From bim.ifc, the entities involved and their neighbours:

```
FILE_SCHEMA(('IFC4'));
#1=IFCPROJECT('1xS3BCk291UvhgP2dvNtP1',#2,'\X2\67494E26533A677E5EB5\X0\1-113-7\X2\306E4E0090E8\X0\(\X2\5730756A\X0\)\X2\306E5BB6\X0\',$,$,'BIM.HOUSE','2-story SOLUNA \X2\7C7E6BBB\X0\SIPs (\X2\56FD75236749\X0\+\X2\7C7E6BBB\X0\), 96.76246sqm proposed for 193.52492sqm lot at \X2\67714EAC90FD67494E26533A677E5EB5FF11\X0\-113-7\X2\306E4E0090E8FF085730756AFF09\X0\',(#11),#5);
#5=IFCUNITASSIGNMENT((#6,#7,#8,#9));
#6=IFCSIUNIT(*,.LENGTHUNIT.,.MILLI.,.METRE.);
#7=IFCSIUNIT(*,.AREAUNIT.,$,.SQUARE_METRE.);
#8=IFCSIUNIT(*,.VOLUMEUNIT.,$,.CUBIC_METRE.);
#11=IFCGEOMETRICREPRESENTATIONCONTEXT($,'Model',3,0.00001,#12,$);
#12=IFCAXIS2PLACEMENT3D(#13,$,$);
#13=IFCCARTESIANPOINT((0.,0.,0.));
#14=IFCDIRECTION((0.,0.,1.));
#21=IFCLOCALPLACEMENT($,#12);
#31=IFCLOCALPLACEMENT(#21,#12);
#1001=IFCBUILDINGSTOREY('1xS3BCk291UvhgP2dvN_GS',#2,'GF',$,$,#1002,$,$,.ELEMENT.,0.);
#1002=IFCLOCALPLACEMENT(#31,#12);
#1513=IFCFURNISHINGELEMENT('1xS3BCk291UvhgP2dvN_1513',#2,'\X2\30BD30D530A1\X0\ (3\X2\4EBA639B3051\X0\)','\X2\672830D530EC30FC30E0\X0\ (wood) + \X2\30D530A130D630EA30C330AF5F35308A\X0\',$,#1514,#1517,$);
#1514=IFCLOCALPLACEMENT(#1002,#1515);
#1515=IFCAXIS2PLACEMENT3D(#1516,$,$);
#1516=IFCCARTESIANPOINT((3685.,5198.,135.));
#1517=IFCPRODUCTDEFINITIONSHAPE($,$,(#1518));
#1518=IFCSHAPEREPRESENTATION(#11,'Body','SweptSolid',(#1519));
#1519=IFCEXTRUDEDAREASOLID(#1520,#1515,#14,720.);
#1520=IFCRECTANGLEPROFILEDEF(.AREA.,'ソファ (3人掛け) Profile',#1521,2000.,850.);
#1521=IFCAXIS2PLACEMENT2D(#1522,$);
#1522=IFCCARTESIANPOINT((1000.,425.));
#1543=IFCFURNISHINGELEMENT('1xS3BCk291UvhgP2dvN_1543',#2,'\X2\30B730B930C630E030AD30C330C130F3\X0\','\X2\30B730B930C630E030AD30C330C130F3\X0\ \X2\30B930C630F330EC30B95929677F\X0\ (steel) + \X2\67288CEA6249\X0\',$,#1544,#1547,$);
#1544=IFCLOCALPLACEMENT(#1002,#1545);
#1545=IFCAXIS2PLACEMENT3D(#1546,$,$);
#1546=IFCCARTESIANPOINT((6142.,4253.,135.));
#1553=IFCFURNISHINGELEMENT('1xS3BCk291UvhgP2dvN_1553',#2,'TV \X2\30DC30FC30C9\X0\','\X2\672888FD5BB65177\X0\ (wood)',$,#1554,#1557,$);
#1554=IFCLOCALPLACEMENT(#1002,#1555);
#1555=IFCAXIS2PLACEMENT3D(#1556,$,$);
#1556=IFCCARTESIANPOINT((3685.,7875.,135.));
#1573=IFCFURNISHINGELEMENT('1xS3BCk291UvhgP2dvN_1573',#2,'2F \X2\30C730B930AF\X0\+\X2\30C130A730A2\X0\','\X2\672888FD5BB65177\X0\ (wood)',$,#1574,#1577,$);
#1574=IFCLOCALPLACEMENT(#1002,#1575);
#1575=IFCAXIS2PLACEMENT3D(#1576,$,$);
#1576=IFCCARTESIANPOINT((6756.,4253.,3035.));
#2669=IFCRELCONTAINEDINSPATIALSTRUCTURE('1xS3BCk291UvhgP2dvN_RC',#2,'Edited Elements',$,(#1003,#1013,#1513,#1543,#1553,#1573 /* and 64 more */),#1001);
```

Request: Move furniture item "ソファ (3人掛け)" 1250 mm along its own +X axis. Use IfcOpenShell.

```python
import ifcopenshell
import ifcopenshell.api.geometry
import ifcopenshell.util.placement
import ifcopenshell.util.unit

model = ifcopenshell.open("bim.ifc")
unit_scale = ifcopenshell.util.unit.calculate_unit_scale(model)

item = model.by_guid("1xS3BCk291UvhgP2dvN_1513")
matrix = ifcopenshell.util.placement.get_local_placement(item.ObjectPlacement)
matrix[:3, 3] += matrix[:3, 0] * 1.25 / unit_scale
ifcopenshell.api.geometry.edit_object_placement(model, product=item, matrix=matrix, is_si=False)

print(ifcopenshell.util.placement.get_local_placement(item.ObjectPlacement).round(3) + 0.0)

model.write("bim-out.ifc")
```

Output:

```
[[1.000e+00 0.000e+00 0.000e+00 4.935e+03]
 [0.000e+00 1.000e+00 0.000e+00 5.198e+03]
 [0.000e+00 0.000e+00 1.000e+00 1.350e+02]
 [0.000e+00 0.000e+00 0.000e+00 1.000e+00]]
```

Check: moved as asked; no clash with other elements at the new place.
